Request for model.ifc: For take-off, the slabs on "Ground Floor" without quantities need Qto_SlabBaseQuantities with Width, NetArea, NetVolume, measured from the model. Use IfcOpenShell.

First a look at what the model holds.

```python
import ifcopenshell
import ifcopenshell.util.element
import ifcopenshell.util.unit

model = ifcopenshell.open("model.ifc")
print(model.schema)
for unit_type in ("LENGTHUNIT", "AREAUNIT", "VOLUMEUNIT"):
    print(unit_type, ifcopenshell.util.unit.calculate_unit_scale(model, unit_type))
storey = next(s for s in model.by_type("IfcBuildingStorey") if s.Name == "Ground Floor")
slabs = [e for e in ifcopenshell.util.element.get_decomposition(storey) if e.is_a("IfcSlab")]
for e in sorted(slabs, key=lambda e: e.id()):
    print(e.id(), e.is_a(), e.Name, list(ifcopenshell.util.element.get_psets(e, qtos_only=True)), sep=" | ")
```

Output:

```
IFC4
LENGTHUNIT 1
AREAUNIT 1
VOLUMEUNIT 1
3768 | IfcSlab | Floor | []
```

```python
import ifcopenshell
import ifcopenshell.api.pset
import ifcopenshell.geom
import ifcopenshell.util.element
import ifcopenshell.util.shape
import ifcopenshell.util.unit

model = ifcopenshell.open("model.ifc")
unit_scale = ifcopenshell.util.unit.calculate_unit_scale(model)
area_scale = ifcopenshell.util.unit.calculate_unit_scale(model, "AREAUNIT")
volume_scale = ifcopenshell.util.unit.calculate_unit_scale(model, "VOLUMEUNIT")
settings = ifcopenshell.geom.settings()

storey = next(s for s in model.by_type("IfcBuildingStorey") if s.Name == "Ground Floor")
slabs = [e for e in ifcopenshell.util.element.get_decomposition(storey) if e.is_a("IfcSlab")]

for e in sorted(slabs, key=lambda e: e.id()):
    if ifcopenshell.util.element.get_psets(e, qtos_only=True, should_inherit=False):
        continue
    # Geometry comes back in metres, in the element's own axes.
    shape = ifcopenshell.geom.create_shape(settings, e)
    values = {
        "Width": ifcopenshell.util.shape.get_z(shape.geometry) / unit_scale,
        "NetArea": ifcopenshell.util.shape.get_footprint_area(shape.geometry) / area_scale,
        "NetVolume": ifcopenshell.util.shape.get_volume(shape.geometry) / volume_scale,
    }
    qto = ifcopenshell.api.pset.add_qto(model, product=e, name="Qto_SlabBaseQuantities")
    ifcopenshell.api.pset.edit_qto(model, qto=qto, properties=values)
    print(e.id(), {k: round(v, 3) for k, v in values.items()})

model.write("model_rev.ifc")
```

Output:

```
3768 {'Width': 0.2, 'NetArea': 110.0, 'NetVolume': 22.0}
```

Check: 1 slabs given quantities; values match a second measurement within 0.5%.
